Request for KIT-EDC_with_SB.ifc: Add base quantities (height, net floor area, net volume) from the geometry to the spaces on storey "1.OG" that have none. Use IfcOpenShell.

First a look at what the model holds.

```python
import ifcopenshell
import ifcopenshell.util.element
import ifcopenshell.util.unit

model = ifcopenshell.open("KIT-EDC_with_SB.ifc")
print(model.schema)
for unit_type in ("LENGTHUNIT", "AREAUNIT", "VOLUMEUNIT"):
    print(unit_type, ifcopenshell.util.unit.calculate_unit_scale(model, unit_type))
storey = next(s for s in model.by_type("IfcBuildingStorey") if s.Name == "1.OG")
spaces = [e for e in ifcopenshell.util.element.get_decomposition(storey) if e.is_a("IfcSpace")]
for e in sorted(spaces, key=lambda e: e.id()):
    print(e.id(), e.is_a(), e.Name, list(ifcopenshell.util.element.get_psets(e, qtos_only=True)), sep=" | ")
```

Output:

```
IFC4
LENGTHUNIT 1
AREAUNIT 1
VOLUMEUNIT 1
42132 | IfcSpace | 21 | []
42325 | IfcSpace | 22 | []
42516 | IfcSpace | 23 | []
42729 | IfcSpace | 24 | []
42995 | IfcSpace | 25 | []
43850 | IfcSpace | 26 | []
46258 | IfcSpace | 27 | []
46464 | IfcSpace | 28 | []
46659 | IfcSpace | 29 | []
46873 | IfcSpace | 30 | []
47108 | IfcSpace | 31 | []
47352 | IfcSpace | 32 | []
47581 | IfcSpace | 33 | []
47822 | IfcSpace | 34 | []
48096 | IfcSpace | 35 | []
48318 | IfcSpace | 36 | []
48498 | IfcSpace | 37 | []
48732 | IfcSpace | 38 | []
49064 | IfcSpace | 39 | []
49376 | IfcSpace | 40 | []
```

```python
import ifcopenshell
import ifcopenshell.api.pset
import ifcopenshell.geom
import ifcopenshell.util.element
import ifcopenshell.util.shape
import ifcopenshell.util.unit

model = ifcopenshell.open("KIT-EDC_with_SB.ifc")
unit_scale = ifcopenshell.util.unit.calculate_unit_scale(model)
area_scale = ifcopenshell.util.unit.calculate_unit_scale(model, "AREAUNIT")
volume_scale = ifcopenshell.util.unit.calculate_unit_scale(model, "VOLUMEUNIT")
settings = ifcopenshell.geom.settings()

storey = next(s for s in model.by_type("IfcBuildingStorey") if s.Name == "1.OG")
spaces = [e for e in ifcopenshell.util.element.get_decomposition(storey) if e.is_a("IfcSpace")]

for e in sorted(spaces, key=lambda e: e.id()):
    if ifcopenshell.util.element.get_psets(e, qtos_only=True, should_inherit=False):
        continue
    # Geometry comes back in metres, in the element's own axes.
    shape = ifcopenshell.geom.create_shape(settings, e)
    values = {
        "Height": ifcopenshell.util.shape.get_z(shape.geometry) / unit_scale,
        "NetFloorArea": ifcopenshell.util.shape.get_footprint_area(shape.geometry) / area_scale,
        "NetVolume": ifcopenshell.util.shape.get_volume(shape.geometry) / volume_scale,
    }
    qto = ifcopenshell.api.pset.add_qto(model, product=e, name="Qto_SpaceBaseQuantities")
    ifcopenshell.api.pset.edit_qto(model, qto=qto, properties=values)
    print(e.id(), {k: round(v, 3) for k, v in values.items()})

model.write("KIT-EDC_with_SB_rev.ifc")
```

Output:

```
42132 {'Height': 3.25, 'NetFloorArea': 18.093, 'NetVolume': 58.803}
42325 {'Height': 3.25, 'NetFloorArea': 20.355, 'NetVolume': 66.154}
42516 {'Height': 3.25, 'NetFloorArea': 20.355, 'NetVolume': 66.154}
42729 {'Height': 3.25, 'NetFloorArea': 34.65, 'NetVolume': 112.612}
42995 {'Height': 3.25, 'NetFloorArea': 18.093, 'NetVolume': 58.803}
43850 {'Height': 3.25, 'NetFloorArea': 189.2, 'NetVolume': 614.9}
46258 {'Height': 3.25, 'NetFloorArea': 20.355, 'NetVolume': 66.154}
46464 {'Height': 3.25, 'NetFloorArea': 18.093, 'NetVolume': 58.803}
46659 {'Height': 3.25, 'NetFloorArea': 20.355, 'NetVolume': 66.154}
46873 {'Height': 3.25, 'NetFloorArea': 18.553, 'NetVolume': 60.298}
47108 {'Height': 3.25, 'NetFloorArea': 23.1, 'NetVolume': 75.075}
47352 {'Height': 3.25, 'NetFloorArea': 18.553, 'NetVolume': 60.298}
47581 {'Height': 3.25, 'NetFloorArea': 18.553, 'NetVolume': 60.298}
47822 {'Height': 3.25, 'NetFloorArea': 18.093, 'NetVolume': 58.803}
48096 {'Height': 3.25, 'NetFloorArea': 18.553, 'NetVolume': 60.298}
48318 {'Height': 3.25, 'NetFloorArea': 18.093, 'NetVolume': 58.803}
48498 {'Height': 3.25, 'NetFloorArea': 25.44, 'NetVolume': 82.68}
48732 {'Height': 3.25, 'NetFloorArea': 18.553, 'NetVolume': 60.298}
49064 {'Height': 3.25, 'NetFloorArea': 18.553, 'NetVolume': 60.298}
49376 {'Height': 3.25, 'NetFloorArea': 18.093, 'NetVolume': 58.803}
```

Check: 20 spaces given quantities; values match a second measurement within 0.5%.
